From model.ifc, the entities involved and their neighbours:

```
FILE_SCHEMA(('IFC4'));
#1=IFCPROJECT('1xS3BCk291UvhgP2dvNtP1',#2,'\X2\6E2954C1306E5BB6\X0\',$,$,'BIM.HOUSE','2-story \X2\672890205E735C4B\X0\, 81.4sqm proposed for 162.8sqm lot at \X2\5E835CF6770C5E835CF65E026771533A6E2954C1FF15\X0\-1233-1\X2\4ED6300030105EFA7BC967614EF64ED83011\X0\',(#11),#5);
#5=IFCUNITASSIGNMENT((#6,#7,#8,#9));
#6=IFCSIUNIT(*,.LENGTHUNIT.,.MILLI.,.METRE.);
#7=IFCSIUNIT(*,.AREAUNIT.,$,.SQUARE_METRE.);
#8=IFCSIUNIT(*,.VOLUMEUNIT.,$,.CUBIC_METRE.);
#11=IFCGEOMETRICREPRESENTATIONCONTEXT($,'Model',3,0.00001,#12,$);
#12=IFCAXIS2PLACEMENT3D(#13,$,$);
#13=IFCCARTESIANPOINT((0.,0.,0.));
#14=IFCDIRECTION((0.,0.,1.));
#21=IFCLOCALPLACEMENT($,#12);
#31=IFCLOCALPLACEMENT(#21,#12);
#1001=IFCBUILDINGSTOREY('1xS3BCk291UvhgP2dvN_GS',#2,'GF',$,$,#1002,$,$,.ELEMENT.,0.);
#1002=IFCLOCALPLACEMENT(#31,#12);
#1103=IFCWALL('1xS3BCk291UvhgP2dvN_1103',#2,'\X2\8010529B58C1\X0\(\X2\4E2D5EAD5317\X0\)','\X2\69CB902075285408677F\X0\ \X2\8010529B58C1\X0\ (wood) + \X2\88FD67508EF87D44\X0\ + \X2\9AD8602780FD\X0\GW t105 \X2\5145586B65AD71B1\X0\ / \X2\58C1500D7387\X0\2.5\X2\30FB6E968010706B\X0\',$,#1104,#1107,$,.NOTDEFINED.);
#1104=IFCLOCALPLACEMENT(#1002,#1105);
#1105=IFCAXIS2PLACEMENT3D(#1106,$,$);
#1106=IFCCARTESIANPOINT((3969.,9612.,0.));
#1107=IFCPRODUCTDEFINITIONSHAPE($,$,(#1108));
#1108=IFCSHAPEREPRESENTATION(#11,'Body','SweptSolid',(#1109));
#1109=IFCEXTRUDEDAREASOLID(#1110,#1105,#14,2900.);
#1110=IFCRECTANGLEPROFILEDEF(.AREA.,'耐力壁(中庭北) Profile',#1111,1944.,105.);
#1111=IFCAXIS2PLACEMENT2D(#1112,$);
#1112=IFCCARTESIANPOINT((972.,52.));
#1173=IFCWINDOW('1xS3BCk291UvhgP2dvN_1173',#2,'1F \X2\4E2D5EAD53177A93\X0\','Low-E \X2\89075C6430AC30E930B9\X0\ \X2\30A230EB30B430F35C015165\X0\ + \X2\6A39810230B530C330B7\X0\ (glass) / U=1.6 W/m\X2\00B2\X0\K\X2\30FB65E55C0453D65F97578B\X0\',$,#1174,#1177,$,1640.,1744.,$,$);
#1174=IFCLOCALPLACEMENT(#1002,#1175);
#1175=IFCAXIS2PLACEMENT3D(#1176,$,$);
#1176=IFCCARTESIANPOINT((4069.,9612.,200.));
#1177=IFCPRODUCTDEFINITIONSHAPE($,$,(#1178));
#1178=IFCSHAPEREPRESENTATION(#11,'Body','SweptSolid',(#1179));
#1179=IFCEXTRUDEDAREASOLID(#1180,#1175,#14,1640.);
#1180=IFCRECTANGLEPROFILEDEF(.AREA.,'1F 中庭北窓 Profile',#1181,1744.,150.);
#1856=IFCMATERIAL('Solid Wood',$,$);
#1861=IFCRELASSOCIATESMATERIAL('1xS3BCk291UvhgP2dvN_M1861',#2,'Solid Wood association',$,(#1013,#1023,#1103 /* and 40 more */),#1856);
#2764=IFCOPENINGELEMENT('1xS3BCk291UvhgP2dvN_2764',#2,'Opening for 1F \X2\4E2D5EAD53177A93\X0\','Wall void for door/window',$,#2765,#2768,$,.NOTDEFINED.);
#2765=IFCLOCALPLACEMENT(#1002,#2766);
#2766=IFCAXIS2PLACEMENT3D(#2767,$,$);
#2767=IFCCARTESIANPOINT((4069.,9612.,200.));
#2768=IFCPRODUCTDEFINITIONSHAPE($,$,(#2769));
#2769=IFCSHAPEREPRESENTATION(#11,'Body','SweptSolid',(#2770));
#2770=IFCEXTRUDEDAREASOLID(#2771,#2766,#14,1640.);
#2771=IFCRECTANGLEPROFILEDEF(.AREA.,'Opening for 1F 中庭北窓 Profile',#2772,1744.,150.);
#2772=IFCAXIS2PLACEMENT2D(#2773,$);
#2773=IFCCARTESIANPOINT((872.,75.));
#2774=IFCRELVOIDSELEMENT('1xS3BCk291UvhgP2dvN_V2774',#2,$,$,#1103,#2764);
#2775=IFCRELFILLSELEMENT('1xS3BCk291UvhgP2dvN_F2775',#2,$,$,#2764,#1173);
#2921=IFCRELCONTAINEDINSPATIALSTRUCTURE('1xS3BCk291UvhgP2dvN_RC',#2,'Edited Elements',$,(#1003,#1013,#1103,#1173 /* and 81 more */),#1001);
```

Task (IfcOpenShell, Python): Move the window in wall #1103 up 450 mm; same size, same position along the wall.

```python
import numpy as np
import ifcopenshell
import ifcopenshell.api.geometry
import ifcopenshell.util.placement
import ifcopenshell.util.unit

model = ifcopenshell.open("model.ifc")
unit_scale = ifcopenshell.util.unit.calculate_unit_scale(model)

window = model.by_guid("1xS3BCk291UvhgP2dvN_1173")
opening = window.FillsVoids[0].RelatingOpeningElement
dz = 450.0

shift = np.array([0.0, 0.0, dz])
# The window is not placed relative to its opening, so move both.
for product in (opening, window):
    matrix = ifcopenshell.util.placement.get_local_placement(product.ObjectPlacement)
    matrix[:3, 3] += shift
    ifcopenshell.api.geometry.edit_object_placement(model, product=product, matrix=matrix, is_si=False)

print(f"moved by {dz * unit_scale:+.3f} m")

model.write("model_edited.ifc")
```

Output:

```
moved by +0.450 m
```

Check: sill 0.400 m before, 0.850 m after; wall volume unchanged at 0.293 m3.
